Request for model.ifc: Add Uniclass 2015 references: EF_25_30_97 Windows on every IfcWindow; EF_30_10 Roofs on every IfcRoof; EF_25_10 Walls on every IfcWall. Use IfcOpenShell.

First a look at what the model holds.

```python
import ifcopenshell

model = ifcopenshell.open("model.ifc")
print(model.schema)
print("classifications:", [c.Name for c in model.by_type("IfcClassification")])
for ifc_class in ("IfcDoor", "IfcRoof", "IfcStair", "IfcWall", "IfcWindow"):
    print(ifc_class, len(model.by_type(ifc_class)))
```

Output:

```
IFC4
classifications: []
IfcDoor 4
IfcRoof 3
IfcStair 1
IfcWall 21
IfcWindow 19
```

```python
import ifcopenshell
import ifcopenshell.api.classification

model = ifcopenshell.open("model.ifc")

system = ifcopenshell.api.classification.add_classification(model, classification="Uniclass 2015")

codes = {
    "IfcWindow": ("EF_25_30_97", "Windows"),
    "IfcRoof": ("EF_30_10", "Roofs"),
    "IfcWall": ("EF_25_10", "Walls"),
}
for ifc_class, (code, name) in codes.items():
    products = model.by_type(ifc_class)
    ifcopenshell.api.classification.add_reference(
        model, products=products, classification=system, identification=code, name=name
    )
    print(code, len(products))

model.write("model_v2.ifc")
```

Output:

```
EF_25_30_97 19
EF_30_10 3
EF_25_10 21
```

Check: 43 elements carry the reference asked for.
